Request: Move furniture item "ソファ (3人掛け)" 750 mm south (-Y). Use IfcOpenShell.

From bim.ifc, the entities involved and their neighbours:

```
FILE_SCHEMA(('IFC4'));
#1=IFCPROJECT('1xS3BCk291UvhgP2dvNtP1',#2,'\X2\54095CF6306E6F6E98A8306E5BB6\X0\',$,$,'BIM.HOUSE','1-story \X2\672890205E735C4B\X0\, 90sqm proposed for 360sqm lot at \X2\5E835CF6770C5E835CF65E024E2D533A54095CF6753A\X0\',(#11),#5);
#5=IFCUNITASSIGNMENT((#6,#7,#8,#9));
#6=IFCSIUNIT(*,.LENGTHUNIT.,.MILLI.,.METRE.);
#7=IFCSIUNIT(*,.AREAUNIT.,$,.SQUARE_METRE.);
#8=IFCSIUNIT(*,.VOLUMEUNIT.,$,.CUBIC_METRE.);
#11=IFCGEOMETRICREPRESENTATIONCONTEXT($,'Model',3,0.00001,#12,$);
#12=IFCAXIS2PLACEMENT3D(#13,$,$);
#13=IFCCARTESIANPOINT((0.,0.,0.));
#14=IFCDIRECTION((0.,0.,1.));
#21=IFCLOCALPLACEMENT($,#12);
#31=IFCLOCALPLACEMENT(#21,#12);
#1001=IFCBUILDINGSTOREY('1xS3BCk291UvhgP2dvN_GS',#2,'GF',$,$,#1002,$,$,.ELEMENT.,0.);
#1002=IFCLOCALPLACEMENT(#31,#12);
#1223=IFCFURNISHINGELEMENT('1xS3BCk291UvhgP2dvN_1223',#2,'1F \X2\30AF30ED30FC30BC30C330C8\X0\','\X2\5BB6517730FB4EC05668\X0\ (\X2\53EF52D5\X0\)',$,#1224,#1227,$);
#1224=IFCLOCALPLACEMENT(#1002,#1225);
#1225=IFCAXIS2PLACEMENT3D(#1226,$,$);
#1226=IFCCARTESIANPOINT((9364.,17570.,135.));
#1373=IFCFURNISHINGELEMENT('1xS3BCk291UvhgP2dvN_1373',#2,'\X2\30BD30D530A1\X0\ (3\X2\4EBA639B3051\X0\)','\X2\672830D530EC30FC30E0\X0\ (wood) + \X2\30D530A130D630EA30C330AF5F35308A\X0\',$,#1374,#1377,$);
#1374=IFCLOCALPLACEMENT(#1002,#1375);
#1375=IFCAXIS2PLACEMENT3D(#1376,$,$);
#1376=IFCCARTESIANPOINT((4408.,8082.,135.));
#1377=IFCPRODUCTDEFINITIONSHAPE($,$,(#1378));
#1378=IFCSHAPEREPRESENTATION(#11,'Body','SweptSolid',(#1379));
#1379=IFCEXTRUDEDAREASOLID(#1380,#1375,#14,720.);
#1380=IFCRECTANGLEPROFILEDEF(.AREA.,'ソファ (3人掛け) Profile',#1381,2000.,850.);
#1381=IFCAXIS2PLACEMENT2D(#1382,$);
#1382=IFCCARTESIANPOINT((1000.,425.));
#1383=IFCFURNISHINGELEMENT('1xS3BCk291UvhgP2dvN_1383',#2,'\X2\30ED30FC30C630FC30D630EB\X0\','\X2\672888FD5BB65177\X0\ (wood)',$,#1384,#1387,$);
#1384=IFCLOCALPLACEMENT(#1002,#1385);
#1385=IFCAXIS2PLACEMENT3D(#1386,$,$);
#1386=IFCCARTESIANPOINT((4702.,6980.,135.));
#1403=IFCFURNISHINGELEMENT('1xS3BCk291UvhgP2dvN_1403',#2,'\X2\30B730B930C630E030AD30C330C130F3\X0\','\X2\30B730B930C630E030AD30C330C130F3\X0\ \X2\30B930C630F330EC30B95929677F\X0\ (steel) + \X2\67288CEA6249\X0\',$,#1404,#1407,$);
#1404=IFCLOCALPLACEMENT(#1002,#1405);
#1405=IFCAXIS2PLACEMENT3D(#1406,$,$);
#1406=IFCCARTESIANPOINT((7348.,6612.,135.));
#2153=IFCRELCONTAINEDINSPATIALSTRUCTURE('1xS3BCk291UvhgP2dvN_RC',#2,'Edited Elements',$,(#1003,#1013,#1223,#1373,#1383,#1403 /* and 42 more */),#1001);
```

```python
import ifcopenshell
import ifcopenshell.api.geometry
import ifcopenshell.util.placement
import ifcopenshell.util.unit

model = ifcopenshell.open("bim.ifc")
unit_scale = ifcopenshell.util.unit.calculate_unit_scale(model)

item = model.by_guid("1xS3BCk291UvhgP2dvN_1373")
matrix = ifcopenshell.util.placement.get_local_placement(item.ObjectPlacement)
matrix[1, 3] -= 0.75 / unit_scale
ifcopenshell.api.geometry.edit_object_placement(model, product=item, matrix=matrix, is_si=False)

print(ifcopenshell.util.placement.get_local_placement(item.ObjectPlacement).round(3) + 0.0)

model.write("bim-out.ifc")
```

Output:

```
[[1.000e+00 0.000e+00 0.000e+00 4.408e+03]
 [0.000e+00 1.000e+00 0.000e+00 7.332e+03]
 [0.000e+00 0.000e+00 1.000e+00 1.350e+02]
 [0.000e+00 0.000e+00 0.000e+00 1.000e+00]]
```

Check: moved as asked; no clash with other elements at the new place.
